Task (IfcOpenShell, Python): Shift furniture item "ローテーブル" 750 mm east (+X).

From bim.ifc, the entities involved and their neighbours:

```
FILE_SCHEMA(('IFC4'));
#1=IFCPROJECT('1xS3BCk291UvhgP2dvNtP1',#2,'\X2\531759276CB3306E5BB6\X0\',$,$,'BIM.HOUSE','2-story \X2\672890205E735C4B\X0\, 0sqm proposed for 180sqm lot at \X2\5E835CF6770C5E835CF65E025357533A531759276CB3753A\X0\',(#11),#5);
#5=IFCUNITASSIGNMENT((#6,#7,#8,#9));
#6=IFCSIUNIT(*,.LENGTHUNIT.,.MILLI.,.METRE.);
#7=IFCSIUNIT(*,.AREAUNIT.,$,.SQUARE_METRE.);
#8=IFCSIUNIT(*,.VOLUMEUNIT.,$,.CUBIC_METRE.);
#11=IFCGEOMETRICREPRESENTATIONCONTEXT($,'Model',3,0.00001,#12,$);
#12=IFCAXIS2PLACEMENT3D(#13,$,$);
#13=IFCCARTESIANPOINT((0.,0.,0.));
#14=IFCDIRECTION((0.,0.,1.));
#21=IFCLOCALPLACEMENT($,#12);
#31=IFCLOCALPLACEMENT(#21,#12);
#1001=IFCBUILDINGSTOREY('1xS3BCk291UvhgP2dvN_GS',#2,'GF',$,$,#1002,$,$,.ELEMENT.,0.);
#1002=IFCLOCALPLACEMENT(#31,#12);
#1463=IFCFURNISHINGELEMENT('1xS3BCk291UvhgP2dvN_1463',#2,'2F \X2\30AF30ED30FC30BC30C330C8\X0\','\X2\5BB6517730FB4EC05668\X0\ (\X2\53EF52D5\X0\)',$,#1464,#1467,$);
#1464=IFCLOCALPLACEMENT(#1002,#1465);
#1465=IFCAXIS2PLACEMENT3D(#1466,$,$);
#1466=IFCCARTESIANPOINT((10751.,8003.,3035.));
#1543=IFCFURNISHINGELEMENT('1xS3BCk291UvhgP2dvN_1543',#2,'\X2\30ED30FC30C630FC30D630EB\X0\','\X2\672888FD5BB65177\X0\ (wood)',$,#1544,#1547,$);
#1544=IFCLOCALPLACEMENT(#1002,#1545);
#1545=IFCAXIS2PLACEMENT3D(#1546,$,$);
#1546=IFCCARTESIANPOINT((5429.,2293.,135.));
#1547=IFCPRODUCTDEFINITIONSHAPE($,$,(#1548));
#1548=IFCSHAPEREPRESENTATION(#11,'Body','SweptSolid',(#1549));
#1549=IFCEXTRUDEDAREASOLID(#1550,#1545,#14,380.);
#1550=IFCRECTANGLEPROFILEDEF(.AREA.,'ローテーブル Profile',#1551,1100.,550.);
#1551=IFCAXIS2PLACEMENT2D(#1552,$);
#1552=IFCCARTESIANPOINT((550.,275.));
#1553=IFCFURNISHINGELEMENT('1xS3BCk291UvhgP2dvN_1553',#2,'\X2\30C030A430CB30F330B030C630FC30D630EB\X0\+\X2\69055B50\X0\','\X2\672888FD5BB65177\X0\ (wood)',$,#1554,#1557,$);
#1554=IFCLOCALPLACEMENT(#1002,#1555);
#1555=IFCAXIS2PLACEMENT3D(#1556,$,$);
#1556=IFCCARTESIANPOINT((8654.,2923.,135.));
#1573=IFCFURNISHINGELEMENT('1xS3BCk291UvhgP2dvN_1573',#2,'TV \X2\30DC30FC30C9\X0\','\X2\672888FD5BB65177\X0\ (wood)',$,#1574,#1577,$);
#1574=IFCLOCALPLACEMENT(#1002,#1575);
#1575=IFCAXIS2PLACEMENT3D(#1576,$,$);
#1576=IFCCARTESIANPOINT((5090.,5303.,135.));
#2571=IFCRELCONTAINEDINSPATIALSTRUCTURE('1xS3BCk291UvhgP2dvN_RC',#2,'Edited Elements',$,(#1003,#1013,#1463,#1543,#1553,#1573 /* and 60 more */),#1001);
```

```python
import ifcopenshell
import ifcopenshell.api.geometry
import ifcopenshell.util.placement

model = ifcopenshell.open("bim.ifc")

item = model.by_id(1543)
matrix = ifcopenshell.util.placement.get_local_placement(item.ObjectPlacement)
matrix[0, 3] += 750.0
ifcopenshell.api.geometry.edit_object_placement(model, product=item, matrix=matrix, is_si=False)

print(ifcopenshell.util.placement.get_local_placement(item.ObjectPlacement).round(3) + 0.0)

model.write("bim_updated.ifc")
```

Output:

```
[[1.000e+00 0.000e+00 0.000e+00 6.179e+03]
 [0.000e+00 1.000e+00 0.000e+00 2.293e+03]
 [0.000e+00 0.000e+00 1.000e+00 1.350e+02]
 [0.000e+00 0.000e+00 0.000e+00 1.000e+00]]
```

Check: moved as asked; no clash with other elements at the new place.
